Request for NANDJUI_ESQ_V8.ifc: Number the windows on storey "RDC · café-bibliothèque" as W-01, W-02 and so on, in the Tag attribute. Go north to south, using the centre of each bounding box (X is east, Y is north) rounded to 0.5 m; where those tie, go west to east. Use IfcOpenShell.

First a look at what the model holds.

```python
import ifcopenshell
import ifcopenshell.util.element
import ifcopenshell.util.placement

model = ifcopenshell.open("NANDJUI_ESQ_V8.ifc")
print(model.schema)
storey = next(s for s in model.by_type("IfcBuildingStorey") if s.Name == "RDC · café-bibliothèque")
windows = [e for e in ifcopenshell.util.element.get_decomposition(storey) if e.is_a("IfcWindow")]
for e in sorted(windows, key=lambda e: e.id()):
    origin = ifcopenshell.util.placement.get_local_placement(e.ObjectPlacement)[:3, 3]
    print(e.id(), e.Tag, e.Name, origin.round(2) + 0.0, sep=" | ")
```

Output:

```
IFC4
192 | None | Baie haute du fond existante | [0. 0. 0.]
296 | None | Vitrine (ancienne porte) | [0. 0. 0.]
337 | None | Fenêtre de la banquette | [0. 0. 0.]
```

```python
import ifcopenshell
import ifcopenshell.geom
import ifcopenshell.util.element
import ifcopenshell.util.shape

model = ifcopenshell.open("NANDJUI_ESQ_V8.ifc")
settings = ifcopenshell.geom.settings()
settings.set("use-world-coords", True)


def centre(element):
    shape = ifcopenshell.geom.create_shape(settings, element)
    return ifcopenshell.util.shape.get_bbox_centroid(shape.geometry)


storey = next(s for s in model.by_type("IfcBuildingStorey") if s.Name == "RDC · café-bibliothèque")
windows = [e for e in ifcopenshell.util.element.get_decomposition(storey) if e.is_a("IfcWindow")]

# Insertion points can sit at a corner or the storey origin, so sort by the geometry (in metres).
centres = {e: centre(e) for e in windows}
windows.sort(key=lambda e: (-round(centres[e][1] / 0.5), centres[e][0]))

for i, e in enumerate(windows, start=1):
    number = f"W-{i:02d}"
    e.Tag = number
    print(e.id(), number)

model.write("NANDJUI_ESQ_V8_rev.ifc")
```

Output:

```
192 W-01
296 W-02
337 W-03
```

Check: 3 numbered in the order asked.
